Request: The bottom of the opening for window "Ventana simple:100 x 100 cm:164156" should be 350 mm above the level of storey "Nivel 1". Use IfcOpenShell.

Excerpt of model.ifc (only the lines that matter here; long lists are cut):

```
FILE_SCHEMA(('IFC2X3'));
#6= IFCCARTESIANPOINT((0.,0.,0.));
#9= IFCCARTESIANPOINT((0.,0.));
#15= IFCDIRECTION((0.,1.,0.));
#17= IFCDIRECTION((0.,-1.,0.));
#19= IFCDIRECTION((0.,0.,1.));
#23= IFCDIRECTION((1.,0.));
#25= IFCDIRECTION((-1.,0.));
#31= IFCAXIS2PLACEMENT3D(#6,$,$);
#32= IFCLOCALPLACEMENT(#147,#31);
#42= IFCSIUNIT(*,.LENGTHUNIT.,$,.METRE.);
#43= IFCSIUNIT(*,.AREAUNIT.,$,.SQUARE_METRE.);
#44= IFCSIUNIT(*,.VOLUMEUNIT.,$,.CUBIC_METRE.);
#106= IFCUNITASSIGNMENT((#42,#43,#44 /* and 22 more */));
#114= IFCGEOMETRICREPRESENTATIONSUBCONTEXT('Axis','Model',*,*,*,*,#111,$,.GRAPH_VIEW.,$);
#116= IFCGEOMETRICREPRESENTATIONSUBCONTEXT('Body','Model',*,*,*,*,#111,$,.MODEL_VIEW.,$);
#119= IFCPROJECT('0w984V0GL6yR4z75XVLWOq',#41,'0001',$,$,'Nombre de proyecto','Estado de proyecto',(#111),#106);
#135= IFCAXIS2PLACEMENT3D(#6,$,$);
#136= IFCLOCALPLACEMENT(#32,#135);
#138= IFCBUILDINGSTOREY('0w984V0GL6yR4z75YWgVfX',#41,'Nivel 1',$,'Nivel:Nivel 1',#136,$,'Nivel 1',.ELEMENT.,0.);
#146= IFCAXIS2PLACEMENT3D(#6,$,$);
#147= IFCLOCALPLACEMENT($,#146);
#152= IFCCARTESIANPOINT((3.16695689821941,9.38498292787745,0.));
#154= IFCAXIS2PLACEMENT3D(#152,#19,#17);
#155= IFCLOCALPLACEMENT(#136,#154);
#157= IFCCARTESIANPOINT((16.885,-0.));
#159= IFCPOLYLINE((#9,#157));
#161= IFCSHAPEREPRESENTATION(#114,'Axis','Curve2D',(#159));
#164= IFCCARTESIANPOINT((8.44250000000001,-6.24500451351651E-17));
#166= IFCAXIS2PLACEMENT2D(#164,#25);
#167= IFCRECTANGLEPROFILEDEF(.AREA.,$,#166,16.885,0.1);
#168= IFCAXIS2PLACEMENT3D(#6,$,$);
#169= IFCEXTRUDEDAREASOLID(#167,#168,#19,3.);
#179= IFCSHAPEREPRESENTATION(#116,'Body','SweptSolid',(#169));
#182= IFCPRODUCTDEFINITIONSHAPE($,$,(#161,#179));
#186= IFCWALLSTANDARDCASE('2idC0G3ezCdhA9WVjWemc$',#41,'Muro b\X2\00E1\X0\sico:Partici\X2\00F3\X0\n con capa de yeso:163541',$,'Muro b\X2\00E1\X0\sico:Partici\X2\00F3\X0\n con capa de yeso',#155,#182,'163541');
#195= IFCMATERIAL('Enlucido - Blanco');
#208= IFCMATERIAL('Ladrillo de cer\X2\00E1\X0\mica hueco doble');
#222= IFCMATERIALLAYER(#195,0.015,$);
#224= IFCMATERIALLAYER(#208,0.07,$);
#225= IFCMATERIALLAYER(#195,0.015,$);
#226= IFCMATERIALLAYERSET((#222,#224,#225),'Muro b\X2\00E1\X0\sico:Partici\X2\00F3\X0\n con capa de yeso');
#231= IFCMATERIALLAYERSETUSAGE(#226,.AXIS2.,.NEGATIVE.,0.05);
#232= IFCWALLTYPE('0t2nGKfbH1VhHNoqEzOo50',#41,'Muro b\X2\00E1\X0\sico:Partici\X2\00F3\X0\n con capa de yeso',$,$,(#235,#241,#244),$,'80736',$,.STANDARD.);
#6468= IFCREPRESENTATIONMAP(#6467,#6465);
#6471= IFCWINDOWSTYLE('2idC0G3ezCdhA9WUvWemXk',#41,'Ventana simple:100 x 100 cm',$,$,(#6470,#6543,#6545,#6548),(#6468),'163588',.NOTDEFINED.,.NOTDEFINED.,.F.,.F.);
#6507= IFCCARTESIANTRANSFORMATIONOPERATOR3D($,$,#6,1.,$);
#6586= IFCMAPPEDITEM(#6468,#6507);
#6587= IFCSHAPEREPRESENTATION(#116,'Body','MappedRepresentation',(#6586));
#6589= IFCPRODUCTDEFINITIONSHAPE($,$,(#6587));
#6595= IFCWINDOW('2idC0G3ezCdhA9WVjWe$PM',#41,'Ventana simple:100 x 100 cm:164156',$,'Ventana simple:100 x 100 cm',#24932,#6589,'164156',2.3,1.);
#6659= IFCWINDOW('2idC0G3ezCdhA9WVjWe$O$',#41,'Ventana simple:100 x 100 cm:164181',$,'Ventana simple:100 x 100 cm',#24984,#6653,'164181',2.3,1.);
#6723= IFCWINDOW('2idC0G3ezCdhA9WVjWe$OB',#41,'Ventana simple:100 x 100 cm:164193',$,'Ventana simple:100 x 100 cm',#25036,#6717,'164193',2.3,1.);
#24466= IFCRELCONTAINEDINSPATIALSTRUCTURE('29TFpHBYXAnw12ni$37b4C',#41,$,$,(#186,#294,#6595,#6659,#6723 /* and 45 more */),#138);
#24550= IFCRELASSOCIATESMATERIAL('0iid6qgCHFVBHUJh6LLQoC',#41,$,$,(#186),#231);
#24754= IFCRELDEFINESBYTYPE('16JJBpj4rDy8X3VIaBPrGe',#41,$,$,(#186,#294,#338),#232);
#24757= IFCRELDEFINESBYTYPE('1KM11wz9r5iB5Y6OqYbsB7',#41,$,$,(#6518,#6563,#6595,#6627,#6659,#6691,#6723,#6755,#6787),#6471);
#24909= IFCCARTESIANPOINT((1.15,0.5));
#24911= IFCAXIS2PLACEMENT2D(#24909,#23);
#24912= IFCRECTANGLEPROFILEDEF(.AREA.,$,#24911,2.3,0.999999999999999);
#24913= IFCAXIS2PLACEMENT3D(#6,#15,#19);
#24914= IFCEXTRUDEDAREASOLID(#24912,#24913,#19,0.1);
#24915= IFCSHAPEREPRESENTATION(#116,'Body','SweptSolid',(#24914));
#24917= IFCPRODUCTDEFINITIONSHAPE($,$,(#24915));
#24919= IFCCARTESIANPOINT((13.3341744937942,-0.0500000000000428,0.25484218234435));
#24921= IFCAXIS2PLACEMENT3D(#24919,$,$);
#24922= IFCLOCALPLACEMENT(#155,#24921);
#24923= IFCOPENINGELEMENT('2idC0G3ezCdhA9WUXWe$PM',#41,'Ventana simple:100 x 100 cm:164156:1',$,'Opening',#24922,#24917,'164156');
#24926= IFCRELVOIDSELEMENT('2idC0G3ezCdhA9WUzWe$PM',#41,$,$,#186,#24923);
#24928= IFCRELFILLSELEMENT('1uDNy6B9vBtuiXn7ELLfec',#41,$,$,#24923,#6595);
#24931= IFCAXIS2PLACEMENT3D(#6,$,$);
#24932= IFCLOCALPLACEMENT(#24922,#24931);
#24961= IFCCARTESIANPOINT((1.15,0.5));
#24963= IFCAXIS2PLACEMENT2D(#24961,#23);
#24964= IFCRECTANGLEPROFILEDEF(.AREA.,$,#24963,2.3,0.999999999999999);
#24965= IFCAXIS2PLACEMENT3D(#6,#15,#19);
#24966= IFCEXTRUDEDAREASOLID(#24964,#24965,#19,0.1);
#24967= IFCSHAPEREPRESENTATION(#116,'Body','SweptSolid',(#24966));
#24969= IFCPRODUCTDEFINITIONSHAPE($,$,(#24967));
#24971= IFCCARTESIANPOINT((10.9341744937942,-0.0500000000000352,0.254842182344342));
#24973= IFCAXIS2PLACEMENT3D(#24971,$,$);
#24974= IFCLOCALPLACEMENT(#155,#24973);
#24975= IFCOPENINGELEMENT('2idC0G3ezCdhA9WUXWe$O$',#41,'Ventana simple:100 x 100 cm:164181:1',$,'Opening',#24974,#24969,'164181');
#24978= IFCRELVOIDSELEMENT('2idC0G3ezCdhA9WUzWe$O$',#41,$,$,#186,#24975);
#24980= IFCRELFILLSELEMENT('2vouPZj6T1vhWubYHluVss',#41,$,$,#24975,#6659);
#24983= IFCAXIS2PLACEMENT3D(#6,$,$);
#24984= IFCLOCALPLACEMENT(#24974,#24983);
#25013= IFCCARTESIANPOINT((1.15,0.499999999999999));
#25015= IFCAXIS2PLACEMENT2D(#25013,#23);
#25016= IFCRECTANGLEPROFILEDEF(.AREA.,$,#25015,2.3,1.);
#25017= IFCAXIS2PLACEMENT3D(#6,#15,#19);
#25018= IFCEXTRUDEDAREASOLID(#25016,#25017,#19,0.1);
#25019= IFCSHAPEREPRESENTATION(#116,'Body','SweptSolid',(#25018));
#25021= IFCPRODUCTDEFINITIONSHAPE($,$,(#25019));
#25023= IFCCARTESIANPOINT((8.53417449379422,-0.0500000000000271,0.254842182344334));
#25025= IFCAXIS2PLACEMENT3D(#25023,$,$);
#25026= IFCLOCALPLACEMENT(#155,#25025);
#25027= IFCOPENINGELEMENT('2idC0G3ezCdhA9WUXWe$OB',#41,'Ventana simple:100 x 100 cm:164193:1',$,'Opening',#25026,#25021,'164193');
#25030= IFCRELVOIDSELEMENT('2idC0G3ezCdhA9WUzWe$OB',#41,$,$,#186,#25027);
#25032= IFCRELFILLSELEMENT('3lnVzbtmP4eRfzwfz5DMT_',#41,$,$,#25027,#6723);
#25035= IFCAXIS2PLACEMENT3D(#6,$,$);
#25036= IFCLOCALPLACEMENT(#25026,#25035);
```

```python
import numpy as np
import ifcopenshell
import ifcopenshell.api.geometry
import ifcopenshell.geom
import ifcopenshell.util.element
import ifcopenshell.util.placement
import ifcopenshell.util.shape
import ifcopenshell.util.unit

model = ifcopenshell.open("model.ifc")
unit_scale = ifcopenshell.util.unit.calculate_unit_scale(model)

window = model.by_guid("2idC0G3ezCdhA9WVjWe$PM")
opening = window.FillsVoids[0].RelatingOpeningElement
storey = ifcopenshell.util.element.get_container(window, ifc_class="IfcBuildingStorey")
level = ifcopenshell.util.placement.get_local_placement(storey.ObjectPlacement)[2, 3]

# The opening's origin need not be at the sill, so measure its lowest point.
shape = ifcopenshell.geom.create_shape(ifcopenshell.geom.settings(), opening)
bottom = ifcopenshell.util.shape.get_shape_bottom_elevation(shape, shape.geometry) / unit_scale
dz = level + 0.35 / unit_scale - bottom

shift = np.array([0.0, 0.0, dz])
# The window is placed relative to its opening, so it follows when the opening moves.
matrix = ifcopenshell.util.placement.get_local_placement(opening.ObjectPlacement)
matrix[:3, 3] += shift
ifcopenshell.api.geometry.edit_object_placement(
    model, product=opening, matrix=matrix, is_si=False, should_transform_children=True
)

print(f"moved by {dz * unit_scale:+.3f} m")

model.write("model_edited.ifc")
```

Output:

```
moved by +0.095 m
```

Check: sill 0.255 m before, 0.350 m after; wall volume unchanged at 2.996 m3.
